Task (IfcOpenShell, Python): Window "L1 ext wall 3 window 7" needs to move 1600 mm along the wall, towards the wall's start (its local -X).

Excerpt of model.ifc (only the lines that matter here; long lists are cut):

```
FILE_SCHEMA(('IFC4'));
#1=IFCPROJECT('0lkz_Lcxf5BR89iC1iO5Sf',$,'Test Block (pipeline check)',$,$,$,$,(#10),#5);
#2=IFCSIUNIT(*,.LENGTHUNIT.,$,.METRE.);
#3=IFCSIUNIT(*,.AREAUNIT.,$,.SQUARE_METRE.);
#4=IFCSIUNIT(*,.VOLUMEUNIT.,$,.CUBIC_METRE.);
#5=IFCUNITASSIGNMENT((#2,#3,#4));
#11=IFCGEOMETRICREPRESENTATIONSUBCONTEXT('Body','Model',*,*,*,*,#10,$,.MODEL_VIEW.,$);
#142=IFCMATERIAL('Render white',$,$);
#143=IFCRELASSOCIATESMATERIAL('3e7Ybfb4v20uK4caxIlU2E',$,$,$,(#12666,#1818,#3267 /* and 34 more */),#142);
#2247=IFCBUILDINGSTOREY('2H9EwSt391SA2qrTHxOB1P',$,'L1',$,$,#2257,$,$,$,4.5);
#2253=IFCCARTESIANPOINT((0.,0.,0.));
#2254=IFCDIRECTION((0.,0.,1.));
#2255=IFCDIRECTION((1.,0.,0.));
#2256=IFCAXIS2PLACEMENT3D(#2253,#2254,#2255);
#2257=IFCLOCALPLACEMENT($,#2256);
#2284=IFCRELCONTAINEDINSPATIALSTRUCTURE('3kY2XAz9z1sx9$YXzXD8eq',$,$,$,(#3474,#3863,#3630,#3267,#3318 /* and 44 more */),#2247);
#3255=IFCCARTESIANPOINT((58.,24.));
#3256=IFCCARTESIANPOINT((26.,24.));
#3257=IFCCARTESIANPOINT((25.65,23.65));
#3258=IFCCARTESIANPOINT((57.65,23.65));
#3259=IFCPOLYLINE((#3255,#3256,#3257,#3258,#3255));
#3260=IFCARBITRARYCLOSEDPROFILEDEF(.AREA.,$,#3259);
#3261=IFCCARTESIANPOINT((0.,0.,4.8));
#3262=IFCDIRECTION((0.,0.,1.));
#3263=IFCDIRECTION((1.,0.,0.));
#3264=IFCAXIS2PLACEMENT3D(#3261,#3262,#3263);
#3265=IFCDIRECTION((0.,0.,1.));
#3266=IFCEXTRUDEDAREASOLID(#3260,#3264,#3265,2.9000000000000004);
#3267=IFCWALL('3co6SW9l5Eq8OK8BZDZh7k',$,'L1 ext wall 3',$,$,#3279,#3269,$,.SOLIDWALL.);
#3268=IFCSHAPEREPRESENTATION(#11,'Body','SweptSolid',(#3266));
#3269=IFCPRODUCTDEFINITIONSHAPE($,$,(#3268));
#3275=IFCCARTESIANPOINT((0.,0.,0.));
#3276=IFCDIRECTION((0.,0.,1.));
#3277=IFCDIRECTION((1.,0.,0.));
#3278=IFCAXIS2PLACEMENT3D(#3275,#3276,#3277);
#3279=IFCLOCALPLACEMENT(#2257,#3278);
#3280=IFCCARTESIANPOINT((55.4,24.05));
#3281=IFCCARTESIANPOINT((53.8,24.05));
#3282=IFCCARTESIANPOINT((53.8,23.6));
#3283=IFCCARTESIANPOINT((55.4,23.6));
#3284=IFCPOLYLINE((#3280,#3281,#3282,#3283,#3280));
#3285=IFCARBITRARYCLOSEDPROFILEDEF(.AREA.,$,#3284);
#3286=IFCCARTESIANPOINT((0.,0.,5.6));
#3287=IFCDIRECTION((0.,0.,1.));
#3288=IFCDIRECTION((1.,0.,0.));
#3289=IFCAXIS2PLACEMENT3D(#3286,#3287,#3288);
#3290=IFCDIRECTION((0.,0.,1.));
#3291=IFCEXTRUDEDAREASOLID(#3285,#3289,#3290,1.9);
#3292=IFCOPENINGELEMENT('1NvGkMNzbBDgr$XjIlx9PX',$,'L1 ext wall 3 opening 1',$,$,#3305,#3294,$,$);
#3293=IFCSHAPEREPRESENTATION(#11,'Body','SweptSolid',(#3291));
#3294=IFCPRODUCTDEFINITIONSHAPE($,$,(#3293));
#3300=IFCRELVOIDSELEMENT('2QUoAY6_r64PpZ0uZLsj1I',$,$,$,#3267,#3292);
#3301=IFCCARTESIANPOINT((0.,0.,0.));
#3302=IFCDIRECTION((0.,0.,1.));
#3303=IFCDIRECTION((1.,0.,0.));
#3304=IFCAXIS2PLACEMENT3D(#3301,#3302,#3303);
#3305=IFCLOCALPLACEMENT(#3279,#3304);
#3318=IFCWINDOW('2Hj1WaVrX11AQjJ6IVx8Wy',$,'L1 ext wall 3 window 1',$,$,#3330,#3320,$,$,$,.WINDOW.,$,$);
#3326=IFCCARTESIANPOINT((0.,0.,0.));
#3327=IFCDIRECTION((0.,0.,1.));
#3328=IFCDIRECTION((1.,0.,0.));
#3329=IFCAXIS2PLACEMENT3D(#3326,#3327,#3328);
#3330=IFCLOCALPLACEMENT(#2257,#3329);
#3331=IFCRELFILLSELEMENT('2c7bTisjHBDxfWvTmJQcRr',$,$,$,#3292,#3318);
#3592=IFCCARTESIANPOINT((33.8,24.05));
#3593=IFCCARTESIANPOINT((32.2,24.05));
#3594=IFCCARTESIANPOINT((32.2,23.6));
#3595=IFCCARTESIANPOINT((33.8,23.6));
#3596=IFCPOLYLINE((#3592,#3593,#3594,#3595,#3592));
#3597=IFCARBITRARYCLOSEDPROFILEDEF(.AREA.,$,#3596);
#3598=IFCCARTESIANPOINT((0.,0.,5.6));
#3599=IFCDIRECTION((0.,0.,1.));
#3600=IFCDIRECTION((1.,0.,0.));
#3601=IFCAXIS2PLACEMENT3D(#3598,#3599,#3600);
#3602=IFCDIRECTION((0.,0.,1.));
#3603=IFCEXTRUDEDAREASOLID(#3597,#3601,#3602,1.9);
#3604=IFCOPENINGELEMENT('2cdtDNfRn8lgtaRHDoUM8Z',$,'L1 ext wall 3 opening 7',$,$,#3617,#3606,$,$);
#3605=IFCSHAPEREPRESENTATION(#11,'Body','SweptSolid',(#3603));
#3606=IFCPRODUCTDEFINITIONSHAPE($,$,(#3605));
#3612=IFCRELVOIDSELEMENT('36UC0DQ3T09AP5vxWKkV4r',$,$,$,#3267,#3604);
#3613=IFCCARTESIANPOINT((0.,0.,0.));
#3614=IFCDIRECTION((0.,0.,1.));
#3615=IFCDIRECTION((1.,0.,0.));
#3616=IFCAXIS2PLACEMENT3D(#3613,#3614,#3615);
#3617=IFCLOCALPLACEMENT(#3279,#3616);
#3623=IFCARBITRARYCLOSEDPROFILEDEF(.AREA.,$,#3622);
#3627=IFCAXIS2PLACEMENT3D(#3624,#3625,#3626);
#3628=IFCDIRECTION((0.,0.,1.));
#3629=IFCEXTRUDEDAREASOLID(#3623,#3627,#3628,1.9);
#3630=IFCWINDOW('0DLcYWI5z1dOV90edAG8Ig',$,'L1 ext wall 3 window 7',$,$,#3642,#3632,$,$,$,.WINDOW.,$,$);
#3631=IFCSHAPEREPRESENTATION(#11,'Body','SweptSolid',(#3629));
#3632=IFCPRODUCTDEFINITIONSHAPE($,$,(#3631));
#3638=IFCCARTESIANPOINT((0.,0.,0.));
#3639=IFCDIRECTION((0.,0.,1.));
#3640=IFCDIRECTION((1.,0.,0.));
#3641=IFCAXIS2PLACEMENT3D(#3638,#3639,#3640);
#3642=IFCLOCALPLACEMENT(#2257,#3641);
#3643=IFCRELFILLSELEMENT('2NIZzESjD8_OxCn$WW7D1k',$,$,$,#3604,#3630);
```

```python
import ifcopenshell
import ifcopenshell.api.geometry
import ifcopenshell.util.placement
import ifcopenshell.util.unit

model = ifcopenshell.open("model.ifc")
unit_scale = ifcopenshell.util.unit.calculate_unit_scale(model)

window = model.by_guid("0DLcYWI5z1dOV90edAG8Ig")
opening = window.FillsVoids[0].RelatingOpeningElement
wall = opening.VoidsElements[0].RelatingBuildingElement

wall_matrix = ifcopenshell.util.placement.get_local_placement(wall.ObjectPlacement)
shift = wall_matrix[:3, 0] * -1.6 / unit_scale
before = ifcopenshell.util.placement.get_local_placement(window.ObjectPlacement)[:3, 3].copy()

# The window is not placed relative to its opening, so move both.
for product in (opening, window):
    matrix = ifcopenshell.util.placement.get_local_placement(product.ObjectPlacement)
    matrix[:3, 3] += shift
    ifcopenshell.api.geometry.edit_object_placement(model, product=product, matrix=matrix, is_si=False)

after = ifcopenshell.util.placement.get_local_placement(window.ObjectPlacement)[:3, 3]
print("window moved by", (after - before).round(3) + 0.0)

model.write("model_edited.ifc")
```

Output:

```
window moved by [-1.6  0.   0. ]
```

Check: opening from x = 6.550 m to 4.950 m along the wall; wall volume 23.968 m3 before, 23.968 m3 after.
